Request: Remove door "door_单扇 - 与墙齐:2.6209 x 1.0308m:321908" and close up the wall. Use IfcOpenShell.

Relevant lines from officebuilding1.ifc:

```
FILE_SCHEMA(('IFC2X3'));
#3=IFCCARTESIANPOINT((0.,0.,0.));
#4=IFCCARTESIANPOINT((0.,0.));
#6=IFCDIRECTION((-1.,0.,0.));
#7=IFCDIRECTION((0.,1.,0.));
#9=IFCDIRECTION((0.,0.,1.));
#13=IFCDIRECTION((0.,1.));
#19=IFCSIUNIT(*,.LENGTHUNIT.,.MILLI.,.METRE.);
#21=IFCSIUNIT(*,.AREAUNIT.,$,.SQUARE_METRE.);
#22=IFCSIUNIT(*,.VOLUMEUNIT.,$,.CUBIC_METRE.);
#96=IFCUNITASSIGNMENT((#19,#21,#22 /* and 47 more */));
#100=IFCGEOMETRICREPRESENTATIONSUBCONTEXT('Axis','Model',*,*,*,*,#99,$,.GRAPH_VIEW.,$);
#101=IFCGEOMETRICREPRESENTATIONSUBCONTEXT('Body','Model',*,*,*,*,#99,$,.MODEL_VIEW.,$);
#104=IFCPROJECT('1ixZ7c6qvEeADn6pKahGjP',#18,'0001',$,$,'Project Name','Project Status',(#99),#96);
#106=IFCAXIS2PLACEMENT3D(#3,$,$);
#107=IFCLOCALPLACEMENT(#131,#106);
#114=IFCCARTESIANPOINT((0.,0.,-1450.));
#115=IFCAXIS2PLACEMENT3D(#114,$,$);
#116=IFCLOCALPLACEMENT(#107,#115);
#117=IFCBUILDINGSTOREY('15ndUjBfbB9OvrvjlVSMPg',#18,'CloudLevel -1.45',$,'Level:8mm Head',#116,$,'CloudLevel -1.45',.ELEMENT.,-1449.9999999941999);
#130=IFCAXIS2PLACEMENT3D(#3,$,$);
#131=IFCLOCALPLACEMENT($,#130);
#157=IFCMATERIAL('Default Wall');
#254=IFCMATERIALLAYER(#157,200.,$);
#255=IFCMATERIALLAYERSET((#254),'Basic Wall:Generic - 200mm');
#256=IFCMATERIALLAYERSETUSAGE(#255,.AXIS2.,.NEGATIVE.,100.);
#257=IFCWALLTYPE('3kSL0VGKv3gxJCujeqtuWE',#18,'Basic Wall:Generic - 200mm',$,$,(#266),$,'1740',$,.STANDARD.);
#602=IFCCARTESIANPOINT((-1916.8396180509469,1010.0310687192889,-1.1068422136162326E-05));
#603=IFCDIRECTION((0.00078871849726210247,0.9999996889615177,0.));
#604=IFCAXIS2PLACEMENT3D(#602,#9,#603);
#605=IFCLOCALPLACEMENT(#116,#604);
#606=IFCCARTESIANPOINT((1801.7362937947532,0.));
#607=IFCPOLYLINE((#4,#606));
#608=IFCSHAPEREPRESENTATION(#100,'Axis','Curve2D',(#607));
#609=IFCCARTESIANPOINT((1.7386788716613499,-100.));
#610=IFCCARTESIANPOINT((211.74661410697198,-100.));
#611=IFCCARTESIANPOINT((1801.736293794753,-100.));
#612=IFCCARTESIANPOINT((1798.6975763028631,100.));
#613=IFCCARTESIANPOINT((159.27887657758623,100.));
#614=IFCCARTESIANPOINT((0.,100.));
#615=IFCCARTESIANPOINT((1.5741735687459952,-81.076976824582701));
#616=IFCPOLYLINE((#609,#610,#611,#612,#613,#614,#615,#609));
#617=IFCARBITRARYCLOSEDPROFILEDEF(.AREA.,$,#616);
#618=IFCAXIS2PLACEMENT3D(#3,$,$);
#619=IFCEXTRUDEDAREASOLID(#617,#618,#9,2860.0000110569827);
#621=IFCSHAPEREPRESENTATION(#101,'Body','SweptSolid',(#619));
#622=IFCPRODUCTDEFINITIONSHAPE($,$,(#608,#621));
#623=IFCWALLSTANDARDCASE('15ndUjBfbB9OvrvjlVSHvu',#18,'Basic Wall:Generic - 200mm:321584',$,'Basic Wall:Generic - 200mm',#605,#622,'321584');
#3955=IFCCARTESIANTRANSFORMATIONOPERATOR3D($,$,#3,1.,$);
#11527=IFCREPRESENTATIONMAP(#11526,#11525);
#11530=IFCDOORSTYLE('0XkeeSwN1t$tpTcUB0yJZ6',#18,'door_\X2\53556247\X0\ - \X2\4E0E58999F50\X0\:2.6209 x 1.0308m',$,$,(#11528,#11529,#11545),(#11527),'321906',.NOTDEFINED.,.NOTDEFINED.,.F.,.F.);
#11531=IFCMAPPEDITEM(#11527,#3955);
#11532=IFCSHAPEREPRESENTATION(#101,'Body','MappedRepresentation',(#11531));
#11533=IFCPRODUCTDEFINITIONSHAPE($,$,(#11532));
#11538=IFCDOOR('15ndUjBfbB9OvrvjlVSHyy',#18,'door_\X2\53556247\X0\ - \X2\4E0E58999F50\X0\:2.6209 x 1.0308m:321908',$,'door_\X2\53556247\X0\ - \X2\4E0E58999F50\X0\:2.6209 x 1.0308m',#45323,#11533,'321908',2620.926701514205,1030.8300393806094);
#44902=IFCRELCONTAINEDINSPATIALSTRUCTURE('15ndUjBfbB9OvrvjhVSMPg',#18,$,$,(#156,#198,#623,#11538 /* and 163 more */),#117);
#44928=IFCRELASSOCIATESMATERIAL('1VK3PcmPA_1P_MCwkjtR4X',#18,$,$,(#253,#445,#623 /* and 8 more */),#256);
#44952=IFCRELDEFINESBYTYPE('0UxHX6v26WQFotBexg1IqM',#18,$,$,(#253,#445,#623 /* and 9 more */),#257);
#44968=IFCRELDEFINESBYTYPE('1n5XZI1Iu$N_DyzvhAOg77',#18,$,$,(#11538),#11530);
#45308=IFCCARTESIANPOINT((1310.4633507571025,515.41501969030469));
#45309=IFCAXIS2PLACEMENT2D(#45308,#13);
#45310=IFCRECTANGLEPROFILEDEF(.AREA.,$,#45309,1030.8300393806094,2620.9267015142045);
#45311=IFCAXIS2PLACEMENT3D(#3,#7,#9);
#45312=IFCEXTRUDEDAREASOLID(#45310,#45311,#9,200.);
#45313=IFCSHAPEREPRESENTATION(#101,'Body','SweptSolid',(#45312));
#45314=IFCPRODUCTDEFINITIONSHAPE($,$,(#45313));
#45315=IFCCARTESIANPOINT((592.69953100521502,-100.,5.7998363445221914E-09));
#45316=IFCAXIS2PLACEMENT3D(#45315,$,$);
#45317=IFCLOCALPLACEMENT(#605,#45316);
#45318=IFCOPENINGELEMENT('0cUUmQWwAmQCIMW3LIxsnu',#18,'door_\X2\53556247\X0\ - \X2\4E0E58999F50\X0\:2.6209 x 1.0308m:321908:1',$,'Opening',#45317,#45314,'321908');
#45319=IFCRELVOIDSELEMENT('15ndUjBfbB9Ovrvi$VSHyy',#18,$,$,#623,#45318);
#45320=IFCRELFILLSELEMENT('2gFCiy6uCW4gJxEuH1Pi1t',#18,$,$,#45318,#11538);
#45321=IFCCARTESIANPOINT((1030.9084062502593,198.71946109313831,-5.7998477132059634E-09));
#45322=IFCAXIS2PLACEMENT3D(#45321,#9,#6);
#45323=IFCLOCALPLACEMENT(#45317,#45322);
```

```python
import ifcopenshell
import ifcopenshell.api.feature
import ifcopenshell.api.root
import ifcopenshell.geom
import ifcopenshell.util.shape

model = ifcopenshell.open("officebuilding1.ifc")
settings = ifcopenshell.geom.settings()


def volume(element):
    """Net volume in cubic metres, openings subtracted."""
    shape = ifcopenshell.geom.create_shape(settings, element)
    return ifcopenshell.util.shape.get_volume(shape.geometry)


door = model.by_id(11538)
opening = door.FillsVoids[0].RelatingOpeningElement
wall = opening.VoidsElements[0].RelatingBuildingElement
before = volume(wall)

ifcopenshell.api.root.remove_product(model, product=door)
ifcopenshell.api.feature.remove_feature(model, feature=opening)

after = volume(wall)

print(f"wall volume {before:.3f} -> {after:.3f} m3")

model.write("officebuilding1_edited.ifc")
```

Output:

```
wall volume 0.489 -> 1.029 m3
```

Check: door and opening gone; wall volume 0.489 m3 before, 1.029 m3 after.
